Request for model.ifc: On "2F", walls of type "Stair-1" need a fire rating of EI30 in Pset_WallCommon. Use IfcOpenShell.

First a look at what the model holds.

```python
import ifcopenshell
import ifcopenshell.util.element

model = ifcopenshell.open("model.ifc")
print(model.schema)
storey = next(s for s in model.by_type("IfcBuildingStorey") if s.Name == "2F")
walls = [e for e in ifcopenshell.util.element.get_decomposition(storey) if e.is_a("IfcWall")]
seen = {}
for e in walls:
    element_type = ifcopenshell.util.element.get_type(e)
    key = (element_type.Name if element_type != e and element_type else None, ifcopenshell.util.element.get_pset(e, "Pset_WallCommon", "FireRating"))
    seen[key] = seen.get(key, 0) + 1
for (name, value), count in sorted(seen.items(), key=str):
    print(count, "x", name, "|", value)
```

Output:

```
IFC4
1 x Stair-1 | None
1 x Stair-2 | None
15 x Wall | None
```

```python
import ifcopenshell
import ifcopenshell.api.pset
import ifcopenshell.util.element

model = ifcopenshell.open("model.ifc")

storey = next(s for s in model.by_type("IfcBuildingStorey") if s.Name == "2F")
walls = [e for e in ifcopenshell.util.element.get_decomposition(storey) if e.is_a("IfcWall")]

count = 0
for e in walls:
    element_type = ifcopenshell.util.element.get_type(e)
    if element_type in (None, e) or element_type.Name != "Stair-1":
        continue
    # add_pset returns the element's existing set when there is one.
    pset = ifcopenshell.api.pset.add_pset(model, product=e, name="Pset_WallCommon")
    ifcopenshell.api.pset.edit_pset(model, pset=pset, properties={"FireRating": "EI30"})
    count += 1

print(count, "walls updated")

model.write("model_v2.ifc")
```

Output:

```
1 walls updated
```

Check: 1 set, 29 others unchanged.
